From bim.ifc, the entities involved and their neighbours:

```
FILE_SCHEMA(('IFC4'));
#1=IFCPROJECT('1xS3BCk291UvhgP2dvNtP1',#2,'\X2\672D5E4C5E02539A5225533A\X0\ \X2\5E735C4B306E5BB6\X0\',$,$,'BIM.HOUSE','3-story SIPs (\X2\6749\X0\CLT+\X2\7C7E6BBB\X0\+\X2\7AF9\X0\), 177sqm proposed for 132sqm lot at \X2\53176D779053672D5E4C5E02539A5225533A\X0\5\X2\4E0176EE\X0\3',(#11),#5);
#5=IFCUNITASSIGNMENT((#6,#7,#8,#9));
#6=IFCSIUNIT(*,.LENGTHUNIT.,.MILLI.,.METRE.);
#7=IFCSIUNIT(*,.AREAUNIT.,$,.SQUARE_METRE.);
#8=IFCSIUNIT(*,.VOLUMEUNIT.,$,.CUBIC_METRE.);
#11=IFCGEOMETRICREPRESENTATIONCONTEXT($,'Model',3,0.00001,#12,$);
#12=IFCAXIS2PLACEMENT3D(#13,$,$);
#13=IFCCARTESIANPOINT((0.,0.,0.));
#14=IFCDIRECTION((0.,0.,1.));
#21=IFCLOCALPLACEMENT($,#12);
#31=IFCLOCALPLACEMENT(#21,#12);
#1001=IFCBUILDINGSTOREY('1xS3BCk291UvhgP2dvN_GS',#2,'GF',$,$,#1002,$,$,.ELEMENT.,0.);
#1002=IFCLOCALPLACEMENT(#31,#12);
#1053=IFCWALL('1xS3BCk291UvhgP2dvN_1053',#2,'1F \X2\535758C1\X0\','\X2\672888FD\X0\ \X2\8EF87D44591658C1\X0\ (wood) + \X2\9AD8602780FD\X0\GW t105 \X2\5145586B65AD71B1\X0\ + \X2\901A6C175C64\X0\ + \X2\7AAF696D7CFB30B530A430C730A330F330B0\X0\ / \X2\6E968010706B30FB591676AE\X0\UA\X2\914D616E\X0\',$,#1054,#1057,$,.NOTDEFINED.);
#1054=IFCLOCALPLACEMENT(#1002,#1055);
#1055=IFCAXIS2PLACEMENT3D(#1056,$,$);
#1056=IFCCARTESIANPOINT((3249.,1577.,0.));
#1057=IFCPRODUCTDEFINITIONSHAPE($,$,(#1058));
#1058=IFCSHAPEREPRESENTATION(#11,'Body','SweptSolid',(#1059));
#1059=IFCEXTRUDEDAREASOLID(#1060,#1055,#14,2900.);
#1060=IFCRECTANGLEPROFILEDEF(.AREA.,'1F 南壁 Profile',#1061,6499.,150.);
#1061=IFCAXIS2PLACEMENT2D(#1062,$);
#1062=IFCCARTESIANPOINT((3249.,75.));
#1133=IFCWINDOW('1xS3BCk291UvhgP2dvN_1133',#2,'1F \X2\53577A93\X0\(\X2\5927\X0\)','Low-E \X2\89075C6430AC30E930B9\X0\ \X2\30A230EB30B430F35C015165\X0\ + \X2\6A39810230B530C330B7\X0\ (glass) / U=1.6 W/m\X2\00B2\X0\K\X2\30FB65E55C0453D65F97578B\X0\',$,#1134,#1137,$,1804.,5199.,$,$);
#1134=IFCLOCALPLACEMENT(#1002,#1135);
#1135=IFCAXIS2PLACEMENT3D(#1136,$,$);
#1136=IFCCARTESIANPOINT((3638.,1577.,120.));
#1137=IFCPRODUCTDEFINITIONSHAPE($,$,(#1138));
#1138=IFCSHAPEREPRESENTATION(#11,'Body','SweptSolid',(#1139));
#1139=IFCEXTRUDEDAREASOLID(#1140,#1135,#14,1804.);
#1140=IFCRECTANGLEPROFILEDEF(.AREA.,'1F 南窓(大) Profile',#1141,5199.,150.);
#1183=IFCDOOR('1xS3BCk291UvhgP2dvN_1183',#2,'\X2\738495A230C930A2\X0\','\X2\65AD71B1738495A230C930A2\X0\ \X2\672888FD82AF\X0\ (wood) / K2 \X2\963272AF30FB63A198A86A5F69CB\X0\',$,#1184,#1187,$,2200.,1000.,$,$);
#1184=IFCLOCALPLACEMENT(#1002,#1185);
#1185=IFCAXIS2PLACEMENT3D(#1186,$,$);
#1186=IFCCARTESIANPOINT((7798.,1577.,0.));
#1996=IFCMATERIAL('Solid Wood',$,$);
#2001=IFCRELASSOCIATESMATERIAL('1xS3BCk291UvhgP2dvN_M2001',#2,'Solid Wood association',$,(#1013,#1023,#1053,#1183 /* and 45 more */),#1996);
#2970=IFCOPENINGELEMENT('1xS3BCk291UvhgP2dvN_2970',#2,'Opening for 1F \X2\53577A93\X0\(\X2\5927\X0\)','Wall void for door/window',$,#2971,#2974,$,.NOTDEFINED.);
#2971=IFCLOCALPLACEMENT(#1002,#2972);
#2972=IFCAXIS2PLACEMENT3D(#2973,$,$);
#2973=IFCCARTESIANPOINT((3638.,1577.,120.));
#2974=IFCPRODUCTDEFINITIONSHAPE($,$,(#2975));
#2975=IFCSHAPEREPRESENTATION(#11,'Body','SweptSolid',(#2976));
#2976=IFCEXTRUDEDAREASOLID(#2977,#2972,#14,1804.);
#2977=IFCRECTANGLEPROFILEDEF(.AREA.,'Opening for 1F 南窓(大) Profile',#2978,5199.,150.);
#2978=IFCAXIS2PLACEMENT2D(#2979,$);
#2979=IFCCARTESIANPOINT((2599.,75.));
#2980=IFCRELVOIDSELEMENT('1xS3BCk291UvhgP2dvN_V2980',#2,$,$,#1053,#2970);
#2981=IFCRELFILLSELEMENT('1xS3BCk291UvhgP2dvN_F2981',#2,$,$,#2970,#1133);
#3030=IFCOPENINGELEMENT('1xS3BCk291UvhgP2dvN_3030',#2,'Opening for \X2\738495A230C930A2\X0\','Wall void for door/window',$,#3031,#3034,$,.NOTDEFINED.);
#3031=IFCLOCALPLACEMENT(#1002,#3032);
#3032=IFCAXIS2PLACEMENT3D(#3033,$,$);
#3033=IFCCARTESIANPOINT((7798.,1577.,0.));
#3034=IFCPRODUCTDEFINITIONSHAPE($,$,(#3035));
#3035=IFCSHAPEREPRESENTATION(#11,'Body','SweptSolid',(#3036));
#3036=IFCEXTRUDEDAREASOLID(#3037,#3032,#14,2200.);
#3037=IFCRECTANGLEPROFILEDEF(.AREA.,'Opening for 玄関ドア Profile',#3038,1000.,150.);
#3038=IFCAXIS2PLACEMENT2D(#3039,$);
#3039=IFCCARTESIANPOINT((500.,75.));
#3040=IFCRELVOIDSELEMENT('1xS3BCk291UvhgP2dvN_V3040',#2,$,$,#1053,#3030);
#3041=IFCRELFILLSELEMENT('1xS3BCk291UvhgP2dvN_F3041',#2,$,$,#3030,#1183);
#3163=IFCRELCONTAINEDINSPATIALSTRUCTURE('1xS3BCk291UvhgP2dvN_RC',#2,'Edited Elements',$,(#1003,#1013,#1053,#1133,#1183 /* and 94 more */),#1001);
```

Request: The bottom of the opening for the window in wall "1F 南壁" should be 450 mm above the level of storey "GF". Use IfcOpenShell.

```python
import numpy as np
import ifcopenshell
import ifcopenshell.api.geometry
import ifcopenshell.geom
import ifcopenshell.util.element
import ifcopenshell.util.placement
import ifcopenshell.util.shape
import ifcopenshell.util.unit

model = ifcopenshell.open("bim.ifc")
unit_scale = ifcopenshell.util.unit.calculate_unit_scale(model)

window = model.by_guid("1xS3BCk291UvhgP2dvN_1133")
opening = window.FillsVoids[0].RelatingOpeningElement
storey = ifcopenshell.util.element.get_container(window, ifc_class="IfcBuildingStorey")
level = ifcopenshell.util.placement.get_local_placement(storey.ObjectPlacement)[2, 3]

# The opening's origin need not be at the sill, so measure its lowest point.
shape = ifcopenshell.geom.create_shape(ifcopenshell.geom.settings(), opening)
bottom = ifcopenshell.util.shape.get_shape_bottom_elevation(shape, shape.geometry) / unit_scale
dz = level + 450.0 - bottom

shift = np.array([0.0, 0.0, dz])
# The window is not placed relative to its opening, so move both.
for product in (opening, window):
    matrix = ifcopenshell.util.placement.get_local_placement(product.ObjectPlacement)
    matrix[:3, 3] += shift
    ifcopenshell.api.geometry.edit_object_placement(model, product=product, matrix=matrix, is_si=False)

print(f"moved by {dz * unit_scale:+.3f} m")

model.write("bim_edited.ifc")
```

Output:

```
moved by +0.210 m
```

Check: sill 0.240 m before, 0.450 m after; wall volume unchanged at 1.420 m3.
